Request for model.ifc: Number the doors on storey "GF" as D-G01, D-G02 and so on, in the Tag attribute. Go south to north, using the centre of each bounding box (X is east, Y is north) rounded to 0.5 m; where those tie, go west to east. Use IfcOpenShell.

First a look at what the model holds.

```python
import ifcopenshell
import ifcopenshell.util.element
import ifcopenshell.util.placement

model = ifcopenshell.open("model.ifc")
print(model.schema)
storey = next(s for s in model.by_type("IfcBuildingStorey") if s.Name == "GF")
doors = [e for e in ifcopenshell.util.element.get_decomposition(storey) if e.is_a("IfcDoor")]
for e in sorted(doors, key=lambda e: e.id()):
    origin = ifcopenshell.util.placement.get_local_placement(e.ObjectPlacement)[:3, 3]
    print(e.id(), e.Tag, e.Name, origin.round(2) + 0.0, sep=" | ")
```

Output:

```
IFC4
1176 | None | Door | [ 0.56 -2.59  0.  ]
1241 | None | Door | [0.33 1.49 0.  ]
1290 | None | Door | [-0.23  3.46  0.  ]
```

```python
import ifcopenshell
import ifcopenshell.geom
import ifcopenshell.util.element
import ifcopenshell.util.shape

model = ifcopenshell.open("model.ifc")
settings = ifcopenshell.geom.settings()
settings.set("use-world-coords", True)


def centre(element):
    shape = ifcopenshell.geom.create_shape(settings, element)
    return ifcopenshell.util.shape.get_bbox_centroid(shape.geometry)


storey = next(s for s in model.by_type("IfcBuildingStorey") if s.Name == "GF")
doors = [e for e in ifcopenshell.util.element.get_decomposition(storey) if e.is_a("IfcDoor")]

# Insertion points can sit at a corner or the storey origin, so sort by the geometry (in metres).
centres = {e: centre(e) for e in doors}
doors.sort(key=lambda e: (round(centres[e][1] / 0.5), centres[e][0]))

for i, e in enumerate(doors, start=1):
    number = f"D-G{i:02d}"
    e.Tag = number
    print(e.id(), number)

model.write("model_edited.ifc")
```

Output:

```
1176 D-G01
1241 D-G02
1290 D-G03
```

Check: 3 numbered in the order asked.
